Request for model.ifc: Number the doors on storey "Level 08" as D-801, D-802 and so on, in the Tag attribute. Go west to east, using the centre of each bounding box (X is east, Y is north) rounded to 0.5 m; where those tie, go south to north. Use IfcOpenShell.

First a look at what the model holds.

```python
import ifcopenshell
import ifcopenshell.util.element
import ifcopenshell.util.placement

model = ifcopenshell.open("model.ifc")
print(model.schema)
storey = next(s for s in model.by_type("IfcBuildingStorey") if s.Name == "Level 08")
doors = [e for e in ifcopenshell.util.element.get_decomposition(storey) if e.is_a("IfcDoor")]
for e in sorted(doors, key=lambda e: e.id()):
    origin = ifcopenshell.util.placement.get_local_placement(e.ObjectPlacement)[:3, 3]
    print(e.id(), e.Tag, e.Name, origin.round(2) + 0.0, sep=" | ")
```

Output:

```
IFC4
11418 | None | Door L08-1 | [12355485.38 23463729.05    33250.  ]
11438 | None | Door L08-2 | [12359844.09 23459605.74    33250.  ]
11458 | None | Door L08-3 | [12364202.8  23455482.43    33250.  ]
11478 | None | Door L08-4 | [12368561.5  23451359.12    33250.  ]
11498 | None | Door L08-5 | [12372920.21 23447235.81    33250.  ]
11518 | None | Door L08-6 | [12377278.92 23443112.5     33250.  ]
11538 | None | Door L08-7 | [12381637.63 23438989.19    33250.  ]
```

```python
import ifcopenshell
import ifcopenshell.geom
import ifcopenshell.util.element
import ifcopenshell.util.shape

model = ifcopenshell.open("model.ifc")
settings = ifcopenshell.geom.settings()
settings.set("use-world-coords", True)


def centre(element):
    shape = ifcopenshell.geom.create_shape(settings, element)
    return ifcopenshell.util.shape.get_bbox_centroid(shape.geometry)


storey = next(s for s in model.by_type("IfcBuildingStorey") if s.Name == "Level 08")
doors = [e for e in ifcopenshell.util.element.get_decomposition(storey) if e.is_a("IfcDoor")]

# Insertion points can sit at a corner or the storey origin, so sort by the geometry (in metres).
centres = {e: centre(e) for e in doors}
doors.sort(key=lambda e: (round(centres[e][0] / 0.5), centres[e][1]))

for i, e in enumerate(doors, start=1):
    number = f"D-8{i:02d}"
    e.Tag = number
    print(e.id(), number)

model.write("model_rev.ifc")
```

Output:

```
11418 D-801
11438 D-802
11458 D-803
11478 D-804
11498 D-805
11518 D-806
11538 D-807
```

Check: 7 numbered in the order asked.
